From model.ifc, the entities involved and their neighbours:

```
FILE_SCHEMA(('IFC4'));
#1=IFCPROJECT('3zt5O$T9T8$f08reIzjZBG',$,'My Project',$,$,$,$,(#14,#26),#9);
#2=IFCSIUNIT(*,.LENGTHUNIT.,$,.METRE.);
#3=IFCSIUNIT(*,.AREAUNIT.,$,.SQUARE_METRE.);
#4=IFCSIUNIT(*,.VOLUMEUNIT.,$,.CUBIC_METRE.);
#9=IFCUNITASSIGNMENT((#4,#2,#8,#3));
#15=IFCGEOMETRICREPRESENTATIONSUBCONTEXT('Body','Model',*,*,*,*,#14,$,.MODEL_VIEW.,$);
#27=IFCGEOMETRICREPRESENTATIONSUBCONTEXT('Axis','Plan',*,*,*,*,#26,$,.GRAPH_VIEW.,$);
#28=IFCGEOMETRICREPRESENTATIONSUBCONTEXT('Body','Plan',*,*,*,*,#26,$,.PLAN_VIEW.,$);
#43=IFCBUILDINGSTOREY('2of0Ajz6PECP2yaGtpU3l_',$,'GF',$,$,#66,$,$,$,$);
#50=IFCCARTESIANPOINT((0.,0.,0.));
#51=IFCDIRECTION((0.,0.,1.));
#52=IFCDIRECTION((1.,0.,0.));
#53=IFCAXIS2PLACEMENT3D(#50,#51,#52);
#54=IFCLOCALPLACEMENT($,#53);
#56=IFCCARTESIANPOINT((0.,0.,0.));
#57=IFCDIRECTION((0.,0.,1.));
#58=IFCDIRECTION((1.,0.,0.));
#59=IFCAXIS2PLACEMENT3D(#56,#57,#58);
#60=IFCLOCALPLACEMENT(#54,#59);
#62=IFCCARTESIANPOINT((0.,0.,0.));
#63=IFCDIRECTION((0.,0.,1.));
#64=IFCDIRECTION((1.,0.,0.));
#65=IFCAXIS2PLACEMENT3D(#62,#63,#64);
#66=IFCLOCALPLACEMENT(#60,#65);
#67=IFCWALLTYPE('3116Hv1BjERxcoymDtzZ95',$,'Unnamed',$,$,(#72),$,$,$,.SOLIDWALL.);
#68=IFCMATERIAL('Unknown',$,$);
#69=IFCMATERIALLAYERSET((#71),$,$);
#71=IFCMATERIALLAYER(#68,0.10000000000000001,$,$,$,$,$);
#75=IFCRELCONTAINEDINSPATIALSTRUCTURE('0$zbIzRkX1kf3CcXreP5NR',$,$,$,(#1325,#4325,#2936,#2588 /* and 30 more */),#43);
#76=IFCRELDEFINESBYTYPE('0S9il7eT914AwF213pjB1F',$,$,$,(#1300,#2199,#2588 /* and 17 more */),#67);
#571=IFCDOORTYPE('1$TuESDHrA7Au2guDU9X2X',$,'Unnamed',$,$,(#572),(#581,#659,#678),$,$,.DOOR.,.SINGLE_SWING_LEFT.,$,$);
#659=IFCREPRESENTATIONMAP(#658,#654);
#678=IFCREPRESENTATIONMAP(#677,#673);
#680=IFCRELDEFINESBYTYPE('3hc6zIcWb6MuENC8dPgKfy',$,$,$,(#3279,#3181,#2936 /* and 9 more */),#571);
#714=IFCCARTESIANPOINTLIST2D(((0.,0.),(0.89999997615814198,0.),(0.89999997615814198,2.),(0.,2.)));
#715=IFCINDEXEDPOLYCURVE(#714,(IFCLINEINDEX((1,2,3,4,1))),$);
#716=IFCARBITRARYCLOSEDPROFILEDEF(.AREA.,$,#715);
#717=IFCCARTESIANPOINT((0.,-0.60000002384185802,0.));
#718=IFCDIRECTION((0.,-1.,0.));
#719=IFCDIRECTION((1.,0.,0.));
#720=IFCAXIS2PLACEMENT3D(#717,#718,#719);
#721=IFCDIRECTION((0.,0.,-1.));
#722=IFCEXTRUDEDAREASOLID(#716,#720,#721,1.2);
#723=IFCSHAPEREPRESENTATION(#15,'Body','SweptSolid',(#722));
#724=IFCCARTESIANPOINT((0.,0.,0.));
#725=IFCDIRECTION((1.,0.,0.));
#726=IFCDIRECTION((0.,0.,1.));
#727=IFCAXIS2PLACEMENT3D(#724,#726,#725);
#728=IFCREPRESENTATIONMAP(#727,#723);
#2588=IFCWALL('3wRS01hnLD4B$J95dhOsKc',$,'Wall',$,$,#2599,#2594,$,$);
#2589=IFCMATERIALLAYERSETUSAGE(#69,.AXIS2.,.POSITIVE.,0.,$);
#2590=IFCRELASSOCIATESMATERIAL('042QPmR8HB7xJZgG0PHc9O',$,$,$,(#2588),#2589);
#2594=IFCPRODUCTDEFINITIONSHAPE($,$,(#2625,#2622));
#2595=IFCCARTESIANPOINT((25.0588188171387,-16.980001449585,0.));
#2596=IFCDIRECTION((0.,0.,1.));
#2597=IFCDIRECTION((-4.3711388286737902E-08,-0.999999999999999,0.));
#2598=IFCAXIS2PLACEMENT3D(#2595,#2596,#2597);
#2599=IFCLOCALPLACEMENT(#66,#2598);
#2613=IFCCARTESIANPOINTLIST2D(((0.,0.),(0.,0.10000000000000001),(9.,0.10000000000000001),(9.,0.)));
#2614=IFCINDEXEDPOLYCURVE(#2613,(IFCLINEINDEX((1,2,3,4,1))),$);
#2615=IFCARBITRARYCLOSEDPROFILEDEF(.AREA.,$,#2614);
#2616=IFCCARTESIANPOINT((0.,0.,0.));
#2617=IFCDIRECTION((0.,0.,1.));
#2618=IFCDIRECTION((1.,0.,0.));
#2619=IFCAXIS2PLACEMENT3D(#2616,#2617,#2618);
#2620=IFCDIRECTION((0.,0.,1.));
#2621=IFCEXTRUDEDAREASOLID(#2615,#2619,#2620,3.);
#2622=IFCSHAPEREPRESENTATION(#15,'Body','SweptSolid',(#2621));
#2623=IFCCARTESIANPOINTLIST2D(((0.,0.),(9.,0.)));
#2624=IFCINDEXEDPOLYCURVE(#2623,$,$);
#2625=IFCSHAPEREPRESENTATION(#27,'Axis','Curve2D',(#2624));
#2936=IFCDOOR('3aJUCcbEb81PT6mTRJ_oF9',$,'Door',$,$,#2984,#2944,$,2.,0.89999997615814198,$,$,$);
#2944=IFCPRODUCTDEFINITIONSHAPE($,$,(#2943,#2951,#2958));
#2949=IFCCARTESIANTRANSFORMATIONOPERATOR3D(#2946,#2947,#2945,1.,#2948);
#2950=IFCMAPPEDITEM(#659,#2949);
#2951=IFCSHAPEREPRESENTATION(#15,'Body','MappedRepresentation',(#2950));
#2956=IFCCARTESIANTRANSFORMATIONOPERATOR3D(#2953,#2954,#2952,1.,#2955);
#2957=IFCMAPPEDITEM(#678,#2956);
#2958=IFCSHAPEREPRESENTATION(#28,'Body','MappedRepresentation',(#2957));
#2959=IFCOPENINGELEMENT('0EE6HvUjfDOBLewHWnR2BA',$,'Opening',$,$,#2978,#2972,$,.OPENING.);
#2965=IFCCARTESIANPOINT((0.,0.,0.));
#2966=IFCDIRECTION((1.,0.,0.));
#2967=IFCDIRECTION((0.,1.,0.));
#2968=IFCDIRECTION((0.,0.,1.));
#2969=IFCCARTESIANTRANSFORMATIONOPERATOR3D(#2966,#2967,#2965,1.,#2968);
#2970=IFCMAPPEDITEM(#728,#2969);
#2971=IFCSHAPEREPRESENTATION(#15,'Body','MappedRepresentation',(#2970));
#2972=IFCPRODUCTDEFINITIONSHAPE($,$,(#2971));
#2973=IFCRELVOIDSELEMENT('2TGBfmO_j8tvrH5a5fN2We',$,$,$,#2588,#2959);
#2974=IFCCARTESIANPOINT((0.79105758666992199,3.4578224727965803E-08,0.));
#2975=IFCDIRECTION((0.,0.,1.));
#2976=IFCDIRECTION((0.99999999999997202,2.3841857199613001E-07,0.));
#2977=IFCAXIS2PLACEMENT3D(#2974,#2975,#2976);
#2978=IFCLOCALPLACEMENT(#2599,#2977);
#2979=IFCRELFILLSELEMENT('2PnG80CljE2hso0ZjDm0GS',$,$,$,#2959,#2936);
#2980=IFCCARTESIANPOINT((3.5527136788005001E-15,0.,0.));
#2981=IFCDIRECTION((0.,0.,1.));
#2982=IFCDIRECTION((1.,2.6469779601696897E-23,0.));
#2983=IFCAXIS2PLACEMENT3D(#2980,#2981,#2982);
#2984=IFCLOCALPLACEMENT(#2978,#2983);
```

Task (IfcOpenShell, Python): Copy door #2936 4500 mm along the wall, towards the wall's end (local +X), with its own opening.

```python
import ifcopenshell
import ifcopenshell.api.feature
import ifcopenshell.api.geometry
import ifcopenshell.api.root
import ifcopenshell.geom
import ifcopenshell.util.element
import ifcopenshell.util.placement
import ifcopenshell.util.shape

model = ifcopenshell.open("model.ifc")
settings = ifcopenshell.geom.settings()


def volume(element):
    """Net volume in cubic metres, openings subtracted."""
    shape = ifcopenshell.geom.create_shape(settings, element)
    return ifcopenshell.util.shape.get_volume(shape.geometry)


door = model.by_id(2936)
opening = door.FillsVoids[0].RelatingOpeningElement
wall = opening.VoidsElements[0].RelatingBuildingElement
before = volume(wall)
shift = ifcopenshell.util.placement.get_local_placement(wall.ObjectPlacement)[:3, 0] * 4.5

# copy_class copies the void relationship, type, container and properties, but no geometry.
new_opening = ifcopenshell.api.root.copy_class(model, product=opening)
new_opening.Representation = ifcopenshell.util.element.copy_deep(
    model, opening.Representation, exclude=["IfcGeometricRepresentationContext", "IfcRepresentationMap"]
)
new_door = ifcopenshell.api.root.copy_class(model, product=door)
new_door.Representation = ifcopenshell.util.element.copy_deep(
    model, door.Representation, exclude=["IfcGeometricRepresentationContext", "IfcRepresentationMap"]
)
ifcopenshell.api.feature.add_filling(model, opening=new_opening, element=new_door)

for old, new in ((opening, new_opening), (door, new_door)):
    matrix = ifcopenshell.util.placement.get_local_placement(old.ObjectPlacement)
    matrix[:3, 3] += shift
    ifcopenshell.api.geometry.edit_object_placement(model, product=new, matrix=matrix, is_si=False)

after = volume(wall)

print(f"wall volume {before:.3f} -> {after:.3f} m3")

model.write("model_updated.ifc")
```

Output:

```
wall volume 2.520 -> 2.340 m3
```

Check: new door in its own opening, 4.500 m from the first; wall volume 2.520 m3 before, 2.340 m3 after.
